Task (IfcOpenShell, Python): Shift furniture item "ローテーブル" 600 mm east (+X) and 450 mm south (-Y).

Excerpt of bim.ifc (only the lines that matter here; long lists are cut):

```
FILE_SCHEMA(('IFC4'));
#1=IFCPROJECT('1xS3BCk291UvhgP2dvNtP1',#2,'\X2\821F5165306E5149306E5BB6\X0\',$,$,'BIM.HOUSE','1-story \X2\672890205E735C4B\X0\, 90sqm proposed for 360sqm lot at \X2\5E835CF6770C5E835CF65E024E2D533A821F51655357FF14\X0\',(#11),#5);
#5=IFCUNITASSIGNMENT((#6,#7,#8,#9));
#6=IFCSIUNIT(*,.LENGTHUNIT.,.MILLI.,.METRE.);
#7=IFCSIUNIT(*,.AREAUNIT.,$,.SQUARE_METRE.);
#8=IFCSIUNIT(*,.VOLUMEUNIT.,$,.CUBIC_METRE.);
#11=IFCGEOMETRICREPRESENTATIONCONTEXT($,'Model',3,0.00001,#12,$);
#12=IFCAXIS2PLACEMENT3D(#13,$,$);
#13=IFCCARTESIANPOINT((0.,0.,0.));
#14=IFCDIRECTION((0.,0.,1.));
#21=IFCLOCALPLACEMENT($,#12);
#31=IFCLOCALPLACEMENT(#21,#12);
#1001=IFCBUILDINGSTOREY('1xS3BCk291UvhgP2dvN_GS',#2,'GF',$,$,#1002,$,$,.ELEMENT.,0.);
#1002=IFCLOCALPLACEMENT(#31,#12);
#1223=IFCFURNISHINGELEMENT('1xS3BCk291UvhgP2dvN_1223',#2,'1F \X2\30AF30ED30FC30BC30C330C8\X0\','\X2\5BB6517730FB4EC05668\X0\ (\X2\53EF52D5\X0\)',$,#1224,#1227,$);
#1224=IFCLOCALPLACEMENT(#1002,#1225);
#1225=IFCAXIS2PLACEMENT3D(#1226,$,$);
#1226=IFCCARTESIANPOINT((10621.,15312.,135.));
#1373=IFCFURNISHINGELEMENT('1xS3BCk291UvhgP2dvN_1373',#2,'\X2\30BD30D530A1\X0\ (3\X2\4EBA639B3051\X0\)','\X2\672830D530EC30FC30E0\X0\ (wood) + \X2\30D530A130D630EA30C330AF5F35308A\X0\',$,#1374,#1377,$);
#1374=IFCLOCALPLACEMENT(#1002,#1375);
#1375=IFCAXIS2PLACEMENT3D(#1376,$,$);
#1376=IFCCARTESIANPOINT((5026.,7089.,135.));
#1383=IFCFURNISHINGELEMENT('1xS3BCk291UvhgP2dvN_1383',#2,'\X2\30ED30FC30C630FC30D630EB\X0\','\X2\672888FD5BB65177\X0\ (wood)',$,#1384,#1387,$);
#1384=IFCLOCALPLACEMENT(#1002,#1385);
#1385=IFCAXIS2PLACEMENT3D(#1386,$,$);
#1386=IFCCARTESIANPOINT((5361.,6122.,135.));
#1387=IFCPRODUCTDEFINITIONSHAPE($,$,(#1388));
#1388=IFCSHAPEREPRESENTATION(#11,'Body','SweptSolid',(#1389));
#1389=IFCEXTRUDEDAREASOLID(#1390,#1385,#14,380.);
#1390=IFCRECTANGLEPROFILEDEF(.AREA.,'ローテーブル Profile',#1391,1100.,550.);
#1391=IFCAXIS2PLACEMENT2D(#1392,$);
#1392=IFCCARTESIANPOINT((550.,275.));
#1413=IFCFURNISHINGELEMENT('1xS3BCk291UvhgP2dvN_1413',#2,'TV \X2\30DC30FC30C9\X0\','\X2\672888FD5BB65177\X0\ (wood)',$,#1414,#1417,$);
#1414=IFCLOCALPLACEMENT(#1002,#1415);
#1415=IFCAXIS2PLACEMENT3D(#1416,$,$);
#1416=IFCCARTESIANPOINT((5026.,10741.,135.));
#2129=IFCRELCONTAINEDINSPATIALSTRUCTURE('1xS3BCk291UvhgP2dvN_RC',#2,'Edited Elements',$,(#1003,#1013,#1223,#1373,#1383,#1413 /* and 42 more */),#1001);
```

```python
import ifcopenshell
import ifcopenshell.api.geometry
import ifcopenshell.util.placement

model = ifcopenshell.open("bim.ifc")

item = model.by_guid("1xS3BCk291UvhgP2dvN_1383")
matrix = ifcopenshell.util.placement.get_local_placement(item.ObjectPlacement)
matrix[0, 3] += 600.0
matrix[1, 3] -= 450.0
ifcopenshell.api.geometry.edit_object_placement(model, product=item, matrix=matrix, is_si=False)

print(ifcopenshell.util.placement.get_local_placement(item.ObjectPlacement).round(3) + 0.0)

model.write("bim-out.ifc")
```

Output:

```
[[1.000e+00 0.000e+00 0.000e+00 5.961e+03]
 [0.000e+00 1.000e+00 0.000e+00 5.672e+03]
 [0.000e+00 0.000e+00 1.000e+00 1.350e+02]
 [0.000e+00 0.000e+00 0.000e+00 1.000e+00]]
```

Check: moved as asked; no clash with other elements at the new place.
